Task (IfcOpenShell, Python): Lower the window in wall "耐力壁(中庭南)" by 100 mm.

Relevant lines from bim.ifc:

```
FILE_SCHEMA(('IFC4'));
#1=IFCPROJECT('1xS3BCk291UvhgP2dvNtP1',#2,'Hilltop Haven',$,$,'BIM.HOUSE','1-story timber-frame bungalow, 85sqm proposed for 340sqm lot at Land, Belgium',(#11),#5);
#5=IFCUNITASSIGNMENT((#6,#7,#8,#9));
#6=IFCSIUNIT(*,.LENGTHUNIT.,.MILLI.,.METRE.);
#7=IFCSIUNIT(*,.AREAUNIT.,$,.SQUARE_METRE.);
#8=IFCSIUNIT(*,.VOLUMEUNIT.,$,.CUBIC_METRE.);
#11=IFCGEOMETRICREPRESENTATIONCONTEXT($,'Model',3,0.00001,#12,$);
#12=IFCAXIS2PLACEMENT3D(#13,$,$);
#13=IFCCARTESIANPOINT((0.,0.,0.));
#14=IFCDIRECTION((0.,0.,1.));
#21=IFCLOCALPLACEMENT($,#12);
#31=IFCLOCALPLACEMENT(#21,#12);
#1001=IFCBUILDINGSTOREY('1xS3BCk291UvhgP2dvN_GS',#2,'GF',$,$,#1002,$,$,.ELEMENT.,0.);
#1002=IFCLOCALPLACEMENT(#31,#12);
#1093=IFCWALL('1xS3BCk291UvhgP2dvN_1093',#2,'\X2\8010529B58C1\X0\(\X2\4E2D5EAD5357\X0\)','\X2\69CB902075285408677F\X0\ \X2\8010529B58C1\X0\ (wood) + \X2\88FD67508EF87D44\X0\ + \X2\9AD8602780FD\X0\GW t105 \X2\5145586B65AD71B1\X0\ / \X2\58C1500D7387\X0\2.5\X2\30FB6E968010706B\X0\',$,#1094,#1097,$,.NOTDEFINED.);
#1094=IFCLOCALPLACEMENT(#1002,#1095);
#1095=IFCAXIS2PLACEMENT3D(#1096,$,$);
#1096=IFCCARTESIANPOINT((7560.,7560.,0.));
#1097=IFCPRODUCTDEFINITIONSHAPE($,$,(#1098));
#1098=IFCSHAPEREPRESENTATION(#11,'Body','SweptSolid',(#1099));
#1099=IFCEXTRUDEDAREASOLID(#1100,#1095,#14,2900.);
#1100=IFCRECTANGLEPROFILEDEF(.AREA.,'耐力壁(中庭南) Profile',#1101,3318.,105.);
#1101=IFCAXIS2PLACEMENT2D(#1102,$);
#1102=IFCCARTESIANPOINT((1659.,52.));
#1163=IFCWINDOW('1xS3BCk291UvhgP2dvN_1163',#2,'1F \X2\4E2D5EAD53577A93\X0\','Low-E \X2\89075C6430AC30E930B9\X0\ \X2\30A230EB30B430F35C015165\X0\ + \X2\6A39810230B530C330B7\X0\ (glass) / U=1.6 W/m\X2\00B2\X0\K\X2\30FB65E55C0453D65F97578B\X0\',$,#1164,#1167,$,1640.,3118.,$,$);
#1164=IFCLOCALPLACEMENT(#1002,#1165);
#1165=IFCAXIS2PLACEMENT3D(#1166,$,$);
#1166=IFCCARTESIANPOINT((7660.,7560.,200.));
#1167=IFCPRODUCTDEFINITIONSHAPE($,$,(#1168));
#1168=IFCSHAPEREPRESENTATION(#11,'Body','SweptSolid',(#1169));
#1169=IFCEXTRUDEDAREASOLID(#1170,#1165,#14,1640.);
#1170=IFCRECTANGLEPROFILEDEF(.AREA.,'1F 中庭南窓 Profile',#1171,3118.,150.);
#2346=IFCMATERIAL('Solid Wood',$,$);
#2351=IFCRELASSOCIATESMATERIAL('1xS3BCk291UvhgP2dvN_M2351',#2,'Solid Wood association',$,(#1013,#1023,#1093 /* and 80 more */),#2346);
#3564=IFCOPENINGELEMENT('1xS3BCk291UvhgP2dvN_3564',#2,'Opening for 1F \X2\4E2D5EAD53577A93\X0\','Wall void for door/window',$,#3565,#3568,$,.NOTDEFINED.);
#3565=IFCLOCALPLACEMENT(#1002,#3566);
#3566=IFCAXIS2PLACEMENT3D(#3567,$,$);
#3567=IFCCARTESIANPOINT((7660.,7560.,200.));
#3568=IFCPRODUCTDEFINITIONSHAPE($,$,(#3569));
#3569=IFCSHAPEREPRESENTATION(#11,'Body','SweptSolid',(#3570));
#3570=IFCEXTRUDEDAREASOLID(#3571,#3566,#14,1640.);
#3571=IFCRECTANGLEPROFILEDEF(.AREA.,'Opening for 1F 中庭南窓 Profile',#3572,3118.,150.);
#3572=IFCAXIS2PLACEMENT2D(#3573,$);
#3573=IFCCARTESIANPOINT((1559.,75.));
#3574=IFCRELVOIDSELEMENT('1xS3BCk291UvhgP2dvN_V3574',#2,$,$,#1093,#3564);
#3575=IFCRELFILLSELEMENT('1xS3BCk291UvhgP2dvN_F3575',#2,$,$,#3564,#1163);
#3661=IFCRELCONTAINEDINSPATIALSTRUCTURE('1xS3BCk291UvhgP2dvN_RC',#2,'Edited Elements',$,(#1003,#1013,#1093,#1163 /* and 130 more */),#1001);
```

```python
import numpy as np
import ifcopenshell
import ifcopenshell.api.geometry
import ifcopenshell.util.placement
import ifcopenshell.util.unit

model = ifcopenshell.open("bim.ifc")
unit_scale = ifcopenshell.util.unit.calculate_unit_scale(model)

window = model.by_guid("1xS3BCk291UvhgP2dvN_1163")
opening = window.FillsVoids[0].RelatingOpeningElement
dz = -0.1 / unit_scale

shift = np.array([0.0, 0.0, dz])
# The window is not placed relative to its opening, so move both.
for product in (opening, window):
    matrix = ifcopenshell.util.placement.get_local_placement(product.ObjectPlacement)
    matrix[:3, 3] += shift
    ifcopenshell.api.geometry.edit_object_placement(model, product=product, matrix=matrix, is_si=False)

print(f"moved by {dz * unit_scale:+.3f} m")

model.write("bim_v2.ifc")
```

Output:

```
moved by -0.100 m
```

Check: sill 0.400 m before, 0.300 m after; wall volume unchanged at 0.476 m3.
